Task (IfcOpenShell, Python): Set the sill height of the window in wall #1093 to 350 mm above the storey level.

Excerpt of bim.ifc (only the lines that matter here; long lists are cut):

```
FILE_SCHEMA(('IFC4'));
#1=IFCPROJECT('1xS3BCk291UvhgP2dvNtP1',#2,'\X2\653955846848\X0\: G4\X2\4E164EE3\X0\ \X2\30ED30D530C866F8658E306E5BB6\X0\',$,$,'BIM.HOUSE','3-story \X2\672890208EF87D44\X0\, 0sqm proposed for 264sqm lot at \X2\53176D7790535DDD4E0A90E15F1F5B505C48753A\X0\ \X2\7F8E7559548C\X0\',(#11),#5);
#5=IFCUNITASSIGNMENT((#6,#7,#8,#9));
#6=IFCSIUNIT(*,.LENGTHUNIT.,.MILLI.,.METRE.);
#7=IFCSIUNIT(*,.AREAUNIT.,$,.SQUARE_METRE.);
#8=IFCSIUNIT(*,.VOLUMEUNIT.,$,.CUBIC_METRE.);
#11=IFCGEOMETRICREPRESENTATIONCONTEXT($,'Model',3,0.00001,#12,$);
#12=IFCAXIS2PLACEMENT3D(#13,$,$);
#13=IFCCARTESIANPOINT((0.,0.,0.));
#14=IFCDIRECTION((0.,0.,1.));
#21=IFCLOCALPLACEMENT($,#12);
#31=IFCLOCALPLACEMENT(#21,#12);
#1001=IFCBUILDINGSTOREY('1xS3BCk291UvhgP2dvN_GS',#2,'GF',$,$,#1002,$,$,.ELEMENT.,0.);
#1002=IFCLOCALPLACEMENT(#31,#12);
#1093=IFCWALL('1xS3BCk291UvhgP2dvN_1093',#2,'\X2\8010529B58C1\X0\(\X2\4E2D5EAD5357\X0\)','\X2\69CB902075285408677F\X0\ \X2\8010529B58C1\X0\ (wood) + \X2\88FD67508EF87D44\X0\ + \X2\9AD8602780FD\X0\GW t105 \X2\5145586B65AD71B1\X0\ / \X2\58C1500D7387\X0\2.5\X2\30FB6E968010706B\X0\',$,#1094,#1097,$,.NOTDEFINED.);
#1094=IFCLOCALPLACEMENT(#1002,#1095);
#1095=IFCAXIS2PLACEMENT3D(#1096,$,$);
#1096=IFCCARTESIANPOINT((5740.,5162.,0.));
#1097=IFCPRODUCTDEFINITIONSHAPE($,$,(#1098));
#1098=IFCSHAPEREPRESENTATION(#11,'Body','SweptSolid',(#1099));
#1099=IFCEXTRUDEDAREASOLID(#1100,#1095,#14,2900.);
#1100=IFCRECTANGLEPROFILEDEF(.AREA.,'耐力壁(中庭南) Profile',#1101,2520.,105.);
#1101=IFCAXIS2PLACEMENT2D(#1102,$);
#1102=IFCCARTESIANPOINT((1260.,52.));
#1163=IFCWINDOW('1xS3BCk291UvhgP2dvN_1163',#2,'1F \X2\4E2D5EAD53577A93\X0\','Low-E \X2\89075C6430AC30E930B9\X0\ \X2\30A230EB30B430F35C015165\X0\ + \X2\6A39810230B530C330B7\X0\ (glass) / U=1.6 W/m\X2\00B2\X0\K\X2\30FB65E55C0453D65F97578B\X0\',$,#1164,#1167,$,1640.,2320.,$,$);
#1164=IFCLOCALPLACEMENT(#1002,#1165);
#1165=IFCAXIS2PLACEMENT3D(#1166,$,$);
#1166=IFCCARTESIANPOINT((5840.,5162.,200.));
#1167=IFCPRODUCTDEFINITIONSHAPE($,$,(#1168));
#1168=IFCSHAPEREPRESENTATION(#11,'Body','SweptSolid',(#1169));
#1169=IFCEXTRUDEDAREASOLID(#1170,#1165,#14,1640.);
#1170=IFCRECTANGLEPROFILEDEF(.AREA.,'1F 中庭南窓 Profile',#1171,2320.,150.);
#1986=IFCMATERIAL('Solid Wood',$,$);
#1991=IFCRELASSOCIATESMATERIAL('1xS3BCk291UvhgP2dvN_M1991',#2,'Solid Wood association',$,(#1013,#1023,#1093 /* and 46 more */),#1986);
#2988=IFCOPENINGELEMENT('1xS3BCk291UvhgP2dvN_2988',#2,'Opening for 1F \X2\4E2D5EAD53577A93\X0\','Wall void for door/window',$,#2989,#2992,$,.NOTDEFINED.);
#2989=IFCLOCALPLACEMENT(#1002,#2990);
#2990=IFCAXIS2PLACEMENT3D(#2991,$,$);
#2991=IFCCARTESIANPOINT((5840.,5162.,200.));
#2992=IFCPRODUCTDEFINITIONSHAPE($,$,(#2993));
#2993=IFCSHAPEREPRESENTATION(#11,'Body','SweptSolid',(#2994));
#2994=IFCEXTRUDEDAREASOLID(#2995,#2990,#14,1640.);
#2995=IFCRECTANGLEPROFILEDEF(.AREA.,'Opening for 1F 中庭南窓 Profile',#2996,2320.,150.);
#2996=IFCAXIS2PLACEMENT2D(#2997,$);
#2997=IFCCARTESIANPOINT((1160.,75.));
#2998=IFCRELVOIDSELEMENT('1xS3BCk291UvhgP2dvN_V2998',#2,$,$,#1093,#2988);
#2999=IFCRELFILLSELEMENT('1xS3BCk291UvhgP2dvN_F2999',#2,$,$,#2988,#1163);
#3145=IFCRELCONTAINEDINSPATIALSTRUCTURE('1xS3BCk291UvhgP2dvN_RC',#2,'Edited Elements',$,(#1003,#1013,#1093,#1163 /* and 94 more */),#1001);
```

```python
import numpy as np
import ifcopenshell
import ifcopenshell.api.geometry
import ifcopenshell.geom
import ifcopenshell.util.element
import ifcopenshell.util.placement
import ifcopenshell.util.shape
import ifcopenshell.util.unit

model = ifcopenshell.open("bim.ifc")
unit_scale = ifcopenshell.util.unit.calculate_unit_scale(model)

window = model.by_guid("1xS3BCk291UvhgP2dvN_1163")
opening = window.FillsVoids[0].RelatingOpeningElement
storey = ifcopenshell.util.element.get_container(window, ifc_class="IfcBuildingStorey")
level = ifcopenshell.util.placement.get_local_placement(storey.ObjectPlacement)[2, 3]

# The opening's origin need not be at the sill, so measure its lowest point.
shape = ifcopenshell.geom.create_shape(ifcopenshell.geom.settings(), opening)
bottom = ifcopenshell.util.shape.get_shape_bottom_elevation(shape, shape.geometry) / unit_scale
dz = level + 0.35 / unit_scale - bottom

shift = np.array([0.0, 0.0, dz])
# The window is not placed relative to its opening, so move both.
for product in (opening, window):
    matrix = ifcopenshell.util.placement.get_local_placement(product.ObjectPlacement)
    matrix[:3, 3] += shift
    ifcopenshell.api.geometry.edit_object_placement(model, product=product, matrix=matrix, is_si=False)

print(f"moved by {dz * unit_scale:+.3f} m")

model.write("bim_v2.ifc")
```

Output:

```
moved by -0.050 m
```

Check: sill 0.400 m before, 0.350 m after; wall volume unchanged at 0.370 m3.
